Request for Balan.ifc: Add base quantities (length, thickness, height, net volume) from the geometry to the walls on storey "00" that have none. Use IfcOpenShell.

First a look at what the model holds.

```python
import ifcopenshell
import ifcopenshell.util.element
import ifcopenshell.util.unit

model = ifcopenshell.open("Balan.ifc")
print(model.schema)
for unit_type in ("LENGTHUNIT", "AREAUNIT", "VOLUMEUNIT"):
    print(unit_type, ifcopenshell.util.unit.calculate_unit_scale(model, unit_type))
storey = next(s for s in model.by_type("IfcBuildingStorey") if s.Name == "00")
walls = [e for e in ifcopenshell.util.element.get_decomposition(storey) if e.is_a("IfcWall")]
for e in sorted(walls, key=lambda e: e.id()):
    print(e.id(), e.is_a(), e.Name, list(ifcopenshell.util.element.get_psets(e, qtos_only=True)), sep=" | ")
```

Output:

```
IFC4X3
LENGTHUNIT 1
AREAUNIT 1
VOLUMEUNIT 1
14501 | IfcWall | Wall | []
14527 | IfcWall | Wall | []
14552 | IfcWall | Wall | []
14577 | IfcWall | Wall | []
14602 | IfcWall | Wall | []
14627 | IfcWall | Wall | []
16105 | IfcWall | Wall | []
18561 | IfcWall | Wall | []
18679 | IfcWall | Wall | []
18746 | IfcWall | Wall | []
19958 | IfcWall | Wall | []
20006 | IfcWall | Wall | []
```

```python
import ifcopenshell
import ifcopenshell.api.pset
import ifcopenshell.geom
import ifcopenshell.util.element
import ifcopenshell.util.shape
import ifcopenshell.util.unit

model = ifcopenshell.open("Balan.ifc")
unit_scale = ifcopenshell.util.unit.calculate_unit_scale(model)
volume_scale = ifcopenshell.util.unit.calculate_unit_scale(model, "VOLUMEUNIT")
settings = ifcopenshell.geom.settings()

storey = next(s for s in model.by_type("IfcBuildingStorey") if s.Name == "00")
walls = [e for e in ifcopenshell.util.element.get_decomposition(storey) if e.is_a("IfcWall")]

for e in sorted(walls, key=lambda e: e.id()):
    if ifcopenshell.util.element.get_psets(e, qtos_only=True, should_inherit=False):
        continue
    # Geometry comes back in metres, in the element's own axes.
    shape = ifcopenshell.geom.create_shape(settings, e)
    values = {
        "Length": ifcopenshell.util.shape.get_x(shape.geometry) / unit_scale,
        "Width": ifcopenshell.util.shape.get_y(shape.geometry) / unit_scale,
        "Height": ifcopenshell.util.shape.get_z(shape.geometry) / unit_scale,
        "NetVolume": ifcopenshell.util.shape.get_volume(shape.geometry) / volume_scale,
    }
    qto = ifcopenshell.api.pset.add_qto(model, product=e, name="Qto_WallBaseQuantities")
    ifcopenshell.api.pset.edit_qto(model, qto=qto, properties=values)
    print(e.id(), {k: round(v, 3) for k, v in values.items()})

model.write("Balan_edited.ifc")
```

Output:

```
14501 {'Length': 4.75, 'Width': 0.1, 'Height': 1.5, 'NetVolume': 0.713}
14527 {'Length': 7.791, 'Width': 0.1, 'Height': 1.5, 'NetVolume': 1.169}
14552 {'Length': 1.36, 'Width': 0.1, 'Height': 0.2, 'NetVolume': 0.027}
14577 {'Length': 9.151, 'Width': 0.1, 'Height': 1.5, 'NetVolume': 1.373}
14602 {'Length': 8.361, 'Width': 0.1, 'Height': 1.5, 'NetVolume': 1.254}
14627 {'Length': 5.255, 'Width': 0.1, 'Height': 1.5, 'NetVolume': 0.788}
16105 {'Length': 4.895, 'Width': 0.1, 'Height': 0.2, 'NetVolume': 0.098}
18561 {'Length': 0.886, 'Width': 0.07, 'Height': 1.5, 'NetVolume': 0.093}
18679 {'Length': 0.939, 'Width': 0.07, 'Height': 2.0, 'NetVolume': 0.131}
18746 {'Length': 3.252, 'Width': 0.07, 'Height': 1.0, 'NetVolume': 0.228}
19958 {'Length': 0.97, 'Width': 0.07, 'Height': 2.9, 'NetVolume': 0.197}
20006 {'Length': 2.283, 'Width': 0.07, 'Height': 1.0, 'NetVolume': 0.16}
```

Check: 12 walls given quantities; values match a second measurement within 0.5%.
